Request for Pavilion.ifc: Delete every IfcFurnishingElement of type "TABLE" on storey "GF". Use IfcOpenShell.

First a look at what the model holds.

```python
import ifcopenshell
import ifcopenshell.util.element

model = ifcopenshell.open("Pavilion.ifc")
print(model.schema)
storey = next(s for s in model.by_type("IfcBuildingStorey") if s.Name == "GF")
furniture = [e for e in ifcopenshell.util.element.get_decomposition(storey) if e.is_a("IfcFurnishingElement")]
seen = {}
for e in furniture:
    element_type = ifcopenshell.util.element.get_type(e)
    name = element_type.Name if element_type not in (None, e) else None
    seen[name] = seen.get(name, 0) + 1
for name, count in sorted(seen.items(), key=str):
    print(count, "x", name)
```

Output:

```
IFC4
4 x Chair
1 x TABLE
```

```python
import ifcopenshell
import ifcopenshell.api.root
import ifcopenshell.util.element

model = ifcopenshell.open("Pavilion.ifc")

storey = next(s for s in model.by_type("IfcBuildingStorey") if s.Name == "GF")
furniture = [e for e in ifcopenshell.util.element.get_decomposition(storey) if e.is_a("IfcFurnishingElement")]
targets = [e for e in furniture if (t := ifcopenshell.util.element.get_type(e)) not in (None, e) and t.Name == "TABLE"]

for e in targets:
    ifcopenshell.api.root.remove_product(model, product=e)
print(len(targets), "removed")

model.write("Pavilion_rev.ifc")
```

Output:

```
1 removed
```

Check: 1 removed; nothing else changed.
